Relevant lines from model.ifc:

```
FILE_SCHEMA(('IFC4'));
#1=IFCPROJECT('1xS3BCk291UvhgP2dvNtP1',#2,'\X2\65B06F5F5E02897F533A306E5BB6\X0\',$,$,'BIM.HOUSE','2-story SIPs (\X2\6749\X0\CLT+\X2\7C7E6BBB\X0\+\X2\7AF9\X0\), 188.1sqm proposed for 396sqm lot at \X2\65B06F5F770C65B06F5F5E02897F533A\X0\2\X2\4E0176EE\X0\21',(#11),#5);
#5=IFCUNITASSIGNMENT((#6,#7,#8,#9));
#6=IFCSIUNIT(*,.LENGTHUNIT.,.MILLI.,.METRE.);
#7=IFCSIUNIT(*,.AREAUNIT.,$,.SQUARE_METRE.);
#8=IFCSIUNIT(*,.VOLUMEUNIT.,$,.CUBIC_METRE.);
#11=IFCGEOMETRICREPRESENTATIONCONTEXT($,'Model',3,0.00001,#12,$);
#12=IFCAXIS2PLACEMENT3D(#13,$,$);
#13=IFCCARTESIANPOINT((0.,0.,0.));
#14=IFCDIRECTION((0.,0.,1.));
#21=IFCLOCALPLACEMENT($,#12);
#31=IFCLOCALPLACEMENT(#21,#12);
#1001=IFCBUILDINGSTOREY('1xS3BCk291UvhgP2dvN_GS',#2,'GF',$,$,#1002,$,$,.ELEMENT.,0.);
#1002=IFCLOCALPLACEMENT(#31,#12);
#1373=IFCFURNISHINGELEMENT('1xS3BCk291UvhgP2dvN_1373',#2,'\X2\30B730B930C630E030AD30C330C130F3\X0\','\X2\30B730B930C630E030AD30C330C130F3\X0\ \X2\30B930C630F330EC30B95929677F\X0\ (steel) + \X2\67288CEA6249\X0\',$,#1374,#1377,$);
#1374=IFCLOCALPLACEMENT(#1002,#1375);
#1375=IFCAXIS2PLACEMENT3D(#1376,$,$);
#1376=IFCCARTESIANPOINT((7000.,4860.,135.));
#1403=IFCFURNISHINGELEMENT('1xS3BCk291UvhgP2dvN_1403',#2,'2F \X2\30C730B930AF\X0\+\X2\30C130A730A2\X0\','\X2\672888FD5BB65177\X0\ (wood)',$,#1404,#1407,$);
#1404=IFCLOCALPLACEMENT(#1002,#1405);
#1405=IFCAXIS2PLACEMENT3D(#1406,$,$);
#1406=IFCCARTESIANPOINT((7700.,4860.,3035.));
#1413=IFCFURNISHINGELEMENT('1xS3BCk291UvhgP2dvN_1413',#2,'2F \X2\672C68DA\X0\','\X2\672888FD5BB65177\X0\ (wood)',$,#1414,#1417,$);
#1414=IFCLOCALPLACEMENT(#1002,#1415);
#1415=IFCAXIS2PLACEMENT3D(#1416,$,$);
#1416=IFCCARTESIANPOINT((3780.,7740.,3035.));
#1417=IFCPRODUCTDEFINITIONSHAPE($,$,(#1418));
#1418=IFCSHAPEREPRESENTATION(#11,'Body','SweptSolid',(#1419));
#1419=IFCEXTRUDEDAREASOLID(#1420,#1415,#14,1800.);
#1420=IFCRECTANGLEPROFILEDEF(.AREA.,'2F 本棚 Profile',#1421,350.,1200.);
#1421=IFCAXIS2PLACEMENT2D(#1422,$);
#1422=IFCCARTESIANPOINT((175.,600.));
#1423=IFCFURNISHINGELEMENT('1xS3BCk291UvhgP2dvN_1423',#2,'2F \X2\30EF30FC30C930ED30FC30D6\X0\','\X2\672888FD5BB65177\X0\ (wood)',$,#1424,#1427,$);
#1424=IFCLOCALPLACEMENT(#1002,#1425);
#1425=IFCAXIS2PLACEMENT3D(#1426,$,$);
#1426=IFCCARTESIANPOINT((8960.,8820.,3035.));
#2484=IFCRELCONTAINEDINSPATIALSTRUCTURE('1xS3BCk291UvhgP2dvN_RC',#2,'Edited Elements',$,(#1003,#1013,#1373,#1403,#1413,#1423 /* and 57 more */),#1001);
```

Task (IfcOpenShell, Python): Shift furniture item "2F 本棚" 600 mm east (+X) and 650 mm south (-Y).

```python
import ifcopenshell
import ifcopenshell.api.geometry
import ifcopenshell.util.placement
import ifcopenshell.util.unit

model = ifcopenshell.open("model.ifc")
unit_scale = ifcopenshell.util.unit.calculate_unit_scale(model)

item = model.by_guid("1xS3BCk291UvhgP2dvN_1413")
matrix = ifcopenshell.util.placement.get_local_placement(item.ObjectPlacement)
matrix[0, 3] += 0.6 / unit_scale
matrix[1, 3] -= 0.65 / unit_scale
ifcopenshell.api.geometry.edit_object_placement(model, product=item, matrix=matrix, is_si=False)

print(ifcopenshell.util.placement.get_local_placement(item.ObjectPlacement).round(3) + 0.0)

model.write("model_rev.ifc")
```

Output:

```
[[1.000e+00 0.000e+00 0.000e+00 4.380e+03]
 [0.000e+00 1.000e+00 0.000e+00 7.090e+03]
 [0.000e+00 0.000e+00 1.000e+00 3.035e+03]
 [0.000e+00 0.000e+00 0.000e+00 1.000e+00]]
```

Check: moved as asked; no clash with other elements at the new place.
